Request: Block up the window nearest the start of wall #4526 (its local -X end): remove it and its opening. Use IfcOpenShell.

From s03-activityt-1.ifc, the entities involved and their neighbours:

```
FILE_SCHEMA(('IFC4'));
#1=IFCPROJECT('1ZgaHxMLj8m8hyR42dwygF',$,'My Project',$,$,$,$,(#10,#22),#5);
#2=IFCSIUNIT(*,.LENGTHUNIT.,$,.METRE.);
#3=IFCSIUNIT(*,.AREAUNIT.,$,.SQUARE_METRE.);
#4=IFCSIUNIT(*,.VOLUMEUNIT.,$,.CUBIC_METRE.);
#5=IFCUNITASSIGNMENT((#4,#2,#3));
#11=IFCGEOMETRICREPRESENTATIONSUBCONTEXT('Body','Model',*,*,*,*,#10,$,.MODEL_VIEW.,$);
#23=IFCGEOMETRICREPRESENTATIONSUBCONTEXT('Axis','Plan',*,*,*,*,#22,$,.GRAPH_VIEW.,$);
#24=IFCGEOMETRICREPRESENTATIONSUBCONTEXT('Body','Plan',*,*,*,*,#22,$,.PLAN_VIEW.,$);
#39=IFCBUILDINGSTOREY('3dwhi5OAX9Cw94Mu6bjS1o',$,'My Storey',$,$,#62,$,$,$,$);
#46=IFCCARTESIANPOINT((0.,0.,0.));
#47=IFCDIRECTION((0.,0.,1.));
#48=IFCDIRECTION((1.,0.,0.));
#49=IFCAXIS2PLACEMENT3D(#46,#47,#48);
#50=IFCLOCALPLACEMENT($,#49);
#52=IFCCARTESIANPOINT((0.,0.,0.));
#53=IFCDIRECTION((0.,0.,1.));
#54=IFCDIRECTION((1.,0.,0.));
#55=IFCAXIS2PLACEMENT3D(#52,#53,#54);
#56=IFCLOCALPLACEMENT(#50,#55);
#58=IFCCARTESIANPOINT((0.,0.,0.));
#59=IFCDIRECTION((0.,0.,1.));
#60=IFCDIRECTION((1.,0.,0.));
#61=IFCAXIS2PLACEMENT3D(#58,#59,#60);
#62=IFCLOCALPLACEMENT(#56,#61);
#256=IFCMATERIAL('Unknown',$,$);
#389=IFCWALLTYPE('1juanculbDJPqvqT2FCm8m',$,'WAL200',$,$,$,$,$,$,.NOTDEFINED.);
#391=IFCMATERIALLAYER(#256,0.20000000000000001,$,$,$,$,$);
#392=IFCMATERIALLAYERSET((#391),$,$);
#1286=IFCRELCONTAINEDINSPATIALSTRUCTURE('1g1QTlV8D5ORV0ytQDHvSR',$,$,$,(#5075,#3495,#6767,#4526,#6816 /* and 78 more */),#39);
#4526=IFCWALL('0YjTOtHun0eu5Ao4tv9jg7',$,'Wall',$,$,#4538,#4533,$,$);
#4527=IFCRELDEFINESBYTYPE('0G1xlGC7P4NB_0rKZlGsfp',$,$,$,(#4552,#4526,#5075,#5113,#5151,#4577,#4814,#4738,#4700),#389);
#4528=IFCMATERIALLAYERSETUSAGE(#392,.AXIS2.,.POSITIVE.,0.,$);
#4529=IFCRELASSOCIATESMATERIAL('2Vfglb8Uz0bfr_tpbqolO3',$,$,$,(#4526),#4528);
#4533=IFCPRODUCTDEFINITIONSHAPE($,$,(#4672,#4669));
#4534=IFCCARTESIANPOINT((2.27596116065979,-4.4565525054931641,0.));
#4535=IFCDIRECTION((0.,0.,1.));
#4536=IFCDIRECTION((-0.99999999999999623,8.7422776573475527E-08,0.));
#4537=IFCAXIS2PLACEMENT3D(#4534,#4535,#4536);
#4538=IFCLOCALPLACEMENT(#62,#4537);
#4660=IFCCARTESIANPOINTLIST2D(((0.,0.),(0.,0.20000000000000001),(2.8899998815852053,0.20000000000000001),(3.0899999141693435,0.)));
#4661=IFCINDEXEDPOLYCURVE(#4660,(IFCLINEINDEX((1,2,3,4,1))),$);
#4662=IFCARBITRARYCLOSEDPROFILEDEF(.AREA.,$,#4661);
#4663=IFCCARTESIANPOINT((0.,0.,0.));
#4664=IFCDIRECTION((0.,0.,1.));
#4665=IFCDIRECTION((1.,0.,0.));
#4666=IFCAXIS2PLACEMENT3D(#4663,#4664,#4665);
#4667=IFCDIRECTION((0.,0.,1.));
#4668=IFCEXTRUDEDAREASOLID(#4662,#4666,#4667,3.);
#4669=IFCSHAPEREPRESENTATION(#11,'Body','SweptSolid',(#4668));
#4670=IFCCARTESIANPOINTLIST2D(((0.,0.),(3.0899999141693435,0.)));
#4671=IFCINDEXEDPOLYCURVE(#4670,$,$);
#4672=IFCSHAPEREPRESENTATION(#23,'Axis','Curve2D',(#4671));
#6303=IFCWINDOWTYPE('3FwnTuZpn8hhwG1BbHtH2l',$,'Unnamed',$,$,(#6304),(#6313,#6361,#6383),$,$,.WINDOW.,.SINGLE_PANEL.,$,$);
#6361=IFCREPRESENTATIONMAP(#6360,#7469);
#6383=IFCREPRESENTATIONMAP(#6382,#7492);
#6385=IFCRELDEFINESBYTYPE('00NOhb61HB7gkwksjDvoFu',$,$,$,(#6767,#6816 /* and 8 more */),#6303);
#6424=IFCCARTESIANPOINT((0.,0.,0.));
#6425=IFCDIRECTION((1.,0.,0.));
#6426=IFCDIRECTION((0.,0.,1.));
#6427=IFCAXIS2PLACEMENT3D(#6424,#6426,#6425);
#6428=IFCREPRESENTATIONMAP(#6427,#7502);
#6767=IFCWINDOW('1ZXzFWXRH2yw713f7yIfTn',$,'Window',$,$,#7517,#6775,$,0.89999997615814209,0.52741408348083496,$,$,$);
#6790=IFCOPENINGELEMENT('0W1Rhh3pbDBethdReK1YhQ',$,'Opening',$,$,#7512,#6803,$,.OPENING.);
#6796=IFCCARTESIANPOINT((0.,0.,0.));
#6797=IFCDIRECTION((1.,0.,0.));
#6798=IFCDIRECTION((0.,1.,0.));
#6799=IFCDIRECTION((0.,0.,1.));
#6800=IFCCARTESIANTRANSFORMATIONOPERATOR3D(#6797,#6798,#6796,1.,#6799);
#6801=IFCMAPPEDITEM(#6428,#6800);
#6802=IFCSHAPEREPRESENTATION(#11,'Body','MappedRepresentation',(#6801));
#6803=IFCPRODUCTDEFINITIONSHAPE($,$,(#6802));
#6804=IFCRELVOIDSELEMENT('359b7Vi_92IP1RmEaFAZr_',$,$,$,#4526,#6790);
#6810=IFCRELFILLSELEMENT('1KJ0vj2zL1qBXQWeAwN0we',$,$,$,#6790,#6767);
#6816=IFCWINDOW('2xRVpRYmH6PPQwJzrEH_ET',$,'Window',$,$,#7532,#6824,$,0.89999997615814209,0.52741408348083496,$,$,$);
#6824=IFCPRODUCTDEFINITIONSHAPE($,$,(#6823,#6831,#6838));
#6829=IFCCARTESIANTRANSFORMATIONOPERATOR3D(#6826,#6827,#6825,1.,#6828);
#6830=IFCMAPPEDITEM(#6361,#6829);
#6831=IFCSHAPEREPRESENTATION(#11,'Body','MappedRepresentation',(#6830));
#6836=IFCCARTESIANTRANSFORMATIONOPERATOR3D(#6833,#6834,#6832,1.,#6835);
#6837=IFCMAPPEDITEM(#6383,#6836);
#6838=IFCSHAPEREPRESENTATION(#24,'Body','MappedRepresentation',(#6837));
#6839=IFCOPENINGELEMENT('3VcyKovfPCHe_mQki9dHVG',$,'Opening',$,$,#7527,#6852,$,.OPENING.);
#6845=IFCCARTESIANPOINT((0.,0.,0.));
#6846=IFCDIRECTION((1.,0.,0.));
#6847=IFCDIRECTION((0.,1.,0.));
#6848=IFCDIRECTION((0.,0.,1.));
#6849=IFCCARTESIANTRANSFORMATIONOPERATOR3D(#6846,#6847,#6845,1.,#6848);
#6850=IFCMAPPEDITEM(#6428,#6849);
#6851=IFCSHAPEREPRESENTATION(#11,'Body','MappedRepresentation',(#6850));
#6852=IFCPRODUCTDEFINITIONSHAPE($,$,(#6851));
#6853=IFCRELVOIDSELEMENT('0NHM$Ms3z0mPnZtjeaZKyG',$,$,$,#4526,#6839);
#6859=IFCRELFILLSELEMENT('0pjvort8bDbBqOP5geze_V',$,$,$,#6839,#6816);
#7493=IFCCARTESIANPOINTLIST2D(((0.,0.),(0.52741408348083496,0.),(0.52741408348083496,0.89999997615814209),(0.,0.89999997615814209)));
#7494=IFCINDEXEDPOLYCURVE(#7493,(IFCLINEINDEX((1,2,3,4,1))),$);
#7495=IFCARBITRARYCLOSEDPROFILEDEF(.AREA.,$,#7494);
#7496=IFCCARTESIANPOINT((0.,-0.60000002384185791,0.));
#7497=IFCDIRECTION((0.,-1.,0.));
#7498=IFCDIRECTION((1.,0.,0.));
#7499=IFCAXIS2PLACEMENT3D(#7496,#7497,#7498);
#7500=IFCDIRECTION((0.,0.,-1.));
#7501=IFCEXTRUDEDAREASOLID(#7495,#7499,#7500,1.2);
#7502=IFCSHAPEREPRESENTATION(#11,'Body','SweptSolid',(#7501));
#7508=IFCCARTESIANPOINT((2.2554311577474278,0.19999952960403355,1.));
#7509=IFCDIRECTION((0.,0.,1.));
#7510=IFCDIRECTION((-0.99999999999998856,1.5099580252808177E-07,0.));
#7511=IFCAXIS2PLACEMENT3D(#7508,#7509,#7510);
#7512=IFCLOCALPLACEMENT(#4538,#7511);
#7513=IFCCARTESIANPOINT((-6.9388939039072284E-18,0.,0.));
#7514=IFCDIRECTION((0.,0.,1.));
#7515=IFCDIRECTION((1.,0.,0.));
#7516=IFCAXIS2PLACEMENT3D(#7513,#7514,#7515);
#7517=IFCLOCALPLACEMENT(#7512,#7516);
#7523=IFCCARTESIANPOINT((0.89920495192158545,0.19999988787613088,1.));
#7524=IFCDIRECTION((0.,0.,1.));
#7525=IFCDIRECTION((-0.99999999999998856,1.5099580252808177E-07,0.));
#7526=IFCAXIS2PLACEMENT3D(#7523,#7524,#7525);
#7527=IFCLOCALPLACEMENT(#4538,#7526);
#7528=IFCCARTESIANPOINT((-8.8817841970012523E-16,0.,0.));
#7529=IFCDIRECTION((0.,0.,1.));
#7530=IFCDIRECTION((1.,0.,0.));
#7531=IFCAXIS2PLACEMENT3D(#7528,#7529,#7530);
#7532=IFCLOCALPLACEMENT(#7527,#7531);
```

```python
import ifcopenshell
import ifcopenshell.api.feature
import ifcopenshell.api.root
import ifcopenshell.geom
import ifcopenshell.util.shape

model = ifcopenshell.open("s03-activityt-1.ifc")
settings = ifcopenshell.geom.settings()


def volume(element):
    """Net volume in cubic metres, openings subtracted."""
    shape = ifcopenshell.geom.create_shape(settings, element)
    return ifcopenshell.util.shape.get_volume(shape.geometry)


window = model.by_guid("2xRVpRYmH6PPQwJzrEH_ET")
opening = window.FillsVoids[0].RelatingOpeningElement
wall = opening.VoidsElements[0].RelatingBuildingElement
before = volume(wall)

ifcopenshell.api.root.remove_product(model, product=window)
ifcopenshell.api.feature.remove_feature(model, feature=opening)

after = volume(wall)

print(f"wall volume {before:.3f} -> {after:.3f} m3")

model.write("s03-activityt-1-out.ifc")
```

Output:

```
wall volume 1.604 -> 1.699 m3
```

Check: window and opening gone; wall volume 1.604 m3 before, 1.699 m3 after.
